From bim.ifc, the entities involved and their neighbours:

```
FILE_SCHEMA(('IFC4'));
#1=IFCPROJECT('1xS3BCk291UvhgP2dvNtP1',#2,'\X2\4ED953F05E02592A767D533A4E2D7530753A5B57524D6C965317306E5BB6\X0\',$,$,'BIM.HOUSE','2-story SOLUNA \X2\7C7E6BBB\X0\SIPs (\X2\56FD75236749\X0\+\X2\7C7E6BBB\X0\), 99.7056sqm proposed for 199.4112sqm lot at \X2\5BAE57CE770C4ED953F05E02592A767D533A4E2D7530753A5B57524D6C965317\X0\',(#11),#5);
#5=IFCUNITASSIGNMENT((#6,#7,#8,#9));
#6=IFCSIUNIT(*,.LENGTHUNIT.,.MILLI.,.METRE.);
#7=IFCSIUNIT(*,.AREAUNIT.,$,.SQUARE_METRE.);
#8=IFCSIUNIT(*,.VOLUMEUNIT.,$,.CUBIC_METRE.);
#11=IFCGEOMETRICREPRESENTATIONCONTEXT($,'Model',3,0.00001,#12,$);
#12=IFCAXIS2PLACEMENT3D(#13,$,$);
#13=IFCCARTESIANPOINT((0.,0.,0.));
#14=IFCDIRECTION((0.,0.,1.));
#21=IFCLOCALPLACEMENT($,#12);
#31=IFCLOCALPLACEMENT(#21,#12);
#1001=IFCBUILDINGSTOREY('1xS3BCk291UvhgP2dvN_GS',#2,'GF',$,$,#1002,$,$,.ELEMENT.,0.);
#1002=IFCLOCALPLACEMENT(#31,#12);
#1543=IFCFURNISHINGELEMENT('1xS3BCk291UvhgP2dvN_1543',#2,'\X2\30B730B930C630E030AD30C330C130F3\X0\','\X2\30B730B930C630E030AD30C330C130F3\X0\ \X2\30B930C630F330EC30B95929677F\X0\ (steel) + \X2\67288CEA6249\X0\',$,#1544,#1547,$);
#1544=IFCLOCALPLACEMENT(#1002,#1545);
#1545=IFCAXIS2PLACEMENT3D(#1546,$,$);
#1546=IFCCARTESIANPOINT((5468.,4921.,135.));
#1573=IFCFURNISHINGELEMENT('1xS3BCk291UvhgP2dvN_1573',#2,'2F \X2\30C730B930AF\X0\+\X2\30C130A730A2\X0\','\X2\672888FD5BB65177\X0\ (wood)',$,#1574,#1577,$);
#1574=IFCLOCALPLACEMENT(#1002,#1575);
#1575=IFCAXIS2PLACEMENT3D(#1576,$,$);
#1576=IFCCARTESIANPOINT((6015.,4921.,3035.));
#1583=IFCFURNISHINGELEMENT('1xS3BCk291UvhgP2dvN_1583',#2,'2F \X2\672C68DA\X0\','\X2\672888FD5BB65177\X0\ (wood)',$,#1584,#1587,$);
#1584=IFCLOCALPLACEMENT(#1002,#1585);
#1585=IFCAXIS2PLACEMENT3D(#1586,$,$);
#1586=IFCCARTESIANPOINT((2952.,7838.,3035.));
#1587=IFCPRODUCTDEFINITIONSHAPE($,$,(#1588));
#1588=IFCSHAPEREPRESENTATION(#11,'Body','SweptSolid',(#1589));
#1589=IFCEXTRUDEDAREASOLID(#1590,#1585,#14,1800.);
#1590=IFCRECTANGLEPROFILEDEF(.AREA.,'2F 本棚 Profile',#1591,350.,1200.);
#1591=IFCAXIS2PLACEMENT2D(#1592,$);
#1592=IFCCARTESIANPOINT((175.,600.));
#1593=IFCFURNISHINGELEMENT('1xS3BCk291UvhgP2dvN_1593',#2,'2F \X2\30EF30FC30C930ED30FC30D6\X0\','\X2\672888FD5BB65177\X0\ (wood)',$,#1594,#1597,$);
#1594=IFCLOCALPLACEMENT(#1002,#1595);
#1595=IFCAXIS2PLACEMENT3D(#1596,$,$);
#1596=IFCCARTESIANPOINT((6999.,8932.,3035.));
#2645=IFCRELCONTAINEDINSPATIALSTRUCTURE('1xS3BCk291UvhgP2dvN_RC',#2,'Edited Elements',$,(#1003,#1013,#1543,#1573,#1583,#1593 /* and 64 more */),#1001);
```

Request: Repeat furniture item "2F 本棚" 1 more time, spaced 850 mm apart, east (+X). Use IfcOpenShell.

```python
import numpy as np
import ifcopenshell
import ifcopenshell.api.geometry
import ifcopenshell.api.root
import ifcopenshell.util.element
import ifcopenshell.util.placement
import ifcopenshell.util.unit

model = ifcopenshell.open("bim.ifc")
unit_scale = ifcopenshell.util.unit.calculate_unit_scale(model)


def reuse_history(source, copy):
    """copy_class also copies each property set's owner history, people and application; keep the originals."""
    for rel in copy.IsDefinedBy:
        if rel.is_a("IfcRelDefinesByProperties") and (history := rel.RelatingPropertyDefinition.OwnerHistory):
            rel.RelatingPropertyDefinition.OwnerHistory = source.OwnerHistory
            ifcopenshell.util.element.remove_deep2(model, history)


source = model.by_id(1583)
base = ifcopenshell.util.placement.get_local_placement(source.ObjectPlacement)
step = np.array([1.0, 0.0, 0.0]) * 0.85 / unit_scale

for i in range(1, 2):
    copy = ifcopenshell.api.root.copy_class(model, product=source)
    copy.Representation = ifcopenshell.util.element.copy_deep(
        model, source.Representation, exclude=["IfcGeometricRepresentationContext", "IfcRepresentationMap"]
    )
    reuse_history(source, copy)
    matrix = base.copy()
    matrix[:3, 3] += i * step
    print("added at", matrix[:3, 3].round(3) + 0.0)
    ifcopenshell.api.geometry.edit_object_placement(model, product=copy, matrix=matrix, is_si=False)

model.write("bim_edited.ifc")
```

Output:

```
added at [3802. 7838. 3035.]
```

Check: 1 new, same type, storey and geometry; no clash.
